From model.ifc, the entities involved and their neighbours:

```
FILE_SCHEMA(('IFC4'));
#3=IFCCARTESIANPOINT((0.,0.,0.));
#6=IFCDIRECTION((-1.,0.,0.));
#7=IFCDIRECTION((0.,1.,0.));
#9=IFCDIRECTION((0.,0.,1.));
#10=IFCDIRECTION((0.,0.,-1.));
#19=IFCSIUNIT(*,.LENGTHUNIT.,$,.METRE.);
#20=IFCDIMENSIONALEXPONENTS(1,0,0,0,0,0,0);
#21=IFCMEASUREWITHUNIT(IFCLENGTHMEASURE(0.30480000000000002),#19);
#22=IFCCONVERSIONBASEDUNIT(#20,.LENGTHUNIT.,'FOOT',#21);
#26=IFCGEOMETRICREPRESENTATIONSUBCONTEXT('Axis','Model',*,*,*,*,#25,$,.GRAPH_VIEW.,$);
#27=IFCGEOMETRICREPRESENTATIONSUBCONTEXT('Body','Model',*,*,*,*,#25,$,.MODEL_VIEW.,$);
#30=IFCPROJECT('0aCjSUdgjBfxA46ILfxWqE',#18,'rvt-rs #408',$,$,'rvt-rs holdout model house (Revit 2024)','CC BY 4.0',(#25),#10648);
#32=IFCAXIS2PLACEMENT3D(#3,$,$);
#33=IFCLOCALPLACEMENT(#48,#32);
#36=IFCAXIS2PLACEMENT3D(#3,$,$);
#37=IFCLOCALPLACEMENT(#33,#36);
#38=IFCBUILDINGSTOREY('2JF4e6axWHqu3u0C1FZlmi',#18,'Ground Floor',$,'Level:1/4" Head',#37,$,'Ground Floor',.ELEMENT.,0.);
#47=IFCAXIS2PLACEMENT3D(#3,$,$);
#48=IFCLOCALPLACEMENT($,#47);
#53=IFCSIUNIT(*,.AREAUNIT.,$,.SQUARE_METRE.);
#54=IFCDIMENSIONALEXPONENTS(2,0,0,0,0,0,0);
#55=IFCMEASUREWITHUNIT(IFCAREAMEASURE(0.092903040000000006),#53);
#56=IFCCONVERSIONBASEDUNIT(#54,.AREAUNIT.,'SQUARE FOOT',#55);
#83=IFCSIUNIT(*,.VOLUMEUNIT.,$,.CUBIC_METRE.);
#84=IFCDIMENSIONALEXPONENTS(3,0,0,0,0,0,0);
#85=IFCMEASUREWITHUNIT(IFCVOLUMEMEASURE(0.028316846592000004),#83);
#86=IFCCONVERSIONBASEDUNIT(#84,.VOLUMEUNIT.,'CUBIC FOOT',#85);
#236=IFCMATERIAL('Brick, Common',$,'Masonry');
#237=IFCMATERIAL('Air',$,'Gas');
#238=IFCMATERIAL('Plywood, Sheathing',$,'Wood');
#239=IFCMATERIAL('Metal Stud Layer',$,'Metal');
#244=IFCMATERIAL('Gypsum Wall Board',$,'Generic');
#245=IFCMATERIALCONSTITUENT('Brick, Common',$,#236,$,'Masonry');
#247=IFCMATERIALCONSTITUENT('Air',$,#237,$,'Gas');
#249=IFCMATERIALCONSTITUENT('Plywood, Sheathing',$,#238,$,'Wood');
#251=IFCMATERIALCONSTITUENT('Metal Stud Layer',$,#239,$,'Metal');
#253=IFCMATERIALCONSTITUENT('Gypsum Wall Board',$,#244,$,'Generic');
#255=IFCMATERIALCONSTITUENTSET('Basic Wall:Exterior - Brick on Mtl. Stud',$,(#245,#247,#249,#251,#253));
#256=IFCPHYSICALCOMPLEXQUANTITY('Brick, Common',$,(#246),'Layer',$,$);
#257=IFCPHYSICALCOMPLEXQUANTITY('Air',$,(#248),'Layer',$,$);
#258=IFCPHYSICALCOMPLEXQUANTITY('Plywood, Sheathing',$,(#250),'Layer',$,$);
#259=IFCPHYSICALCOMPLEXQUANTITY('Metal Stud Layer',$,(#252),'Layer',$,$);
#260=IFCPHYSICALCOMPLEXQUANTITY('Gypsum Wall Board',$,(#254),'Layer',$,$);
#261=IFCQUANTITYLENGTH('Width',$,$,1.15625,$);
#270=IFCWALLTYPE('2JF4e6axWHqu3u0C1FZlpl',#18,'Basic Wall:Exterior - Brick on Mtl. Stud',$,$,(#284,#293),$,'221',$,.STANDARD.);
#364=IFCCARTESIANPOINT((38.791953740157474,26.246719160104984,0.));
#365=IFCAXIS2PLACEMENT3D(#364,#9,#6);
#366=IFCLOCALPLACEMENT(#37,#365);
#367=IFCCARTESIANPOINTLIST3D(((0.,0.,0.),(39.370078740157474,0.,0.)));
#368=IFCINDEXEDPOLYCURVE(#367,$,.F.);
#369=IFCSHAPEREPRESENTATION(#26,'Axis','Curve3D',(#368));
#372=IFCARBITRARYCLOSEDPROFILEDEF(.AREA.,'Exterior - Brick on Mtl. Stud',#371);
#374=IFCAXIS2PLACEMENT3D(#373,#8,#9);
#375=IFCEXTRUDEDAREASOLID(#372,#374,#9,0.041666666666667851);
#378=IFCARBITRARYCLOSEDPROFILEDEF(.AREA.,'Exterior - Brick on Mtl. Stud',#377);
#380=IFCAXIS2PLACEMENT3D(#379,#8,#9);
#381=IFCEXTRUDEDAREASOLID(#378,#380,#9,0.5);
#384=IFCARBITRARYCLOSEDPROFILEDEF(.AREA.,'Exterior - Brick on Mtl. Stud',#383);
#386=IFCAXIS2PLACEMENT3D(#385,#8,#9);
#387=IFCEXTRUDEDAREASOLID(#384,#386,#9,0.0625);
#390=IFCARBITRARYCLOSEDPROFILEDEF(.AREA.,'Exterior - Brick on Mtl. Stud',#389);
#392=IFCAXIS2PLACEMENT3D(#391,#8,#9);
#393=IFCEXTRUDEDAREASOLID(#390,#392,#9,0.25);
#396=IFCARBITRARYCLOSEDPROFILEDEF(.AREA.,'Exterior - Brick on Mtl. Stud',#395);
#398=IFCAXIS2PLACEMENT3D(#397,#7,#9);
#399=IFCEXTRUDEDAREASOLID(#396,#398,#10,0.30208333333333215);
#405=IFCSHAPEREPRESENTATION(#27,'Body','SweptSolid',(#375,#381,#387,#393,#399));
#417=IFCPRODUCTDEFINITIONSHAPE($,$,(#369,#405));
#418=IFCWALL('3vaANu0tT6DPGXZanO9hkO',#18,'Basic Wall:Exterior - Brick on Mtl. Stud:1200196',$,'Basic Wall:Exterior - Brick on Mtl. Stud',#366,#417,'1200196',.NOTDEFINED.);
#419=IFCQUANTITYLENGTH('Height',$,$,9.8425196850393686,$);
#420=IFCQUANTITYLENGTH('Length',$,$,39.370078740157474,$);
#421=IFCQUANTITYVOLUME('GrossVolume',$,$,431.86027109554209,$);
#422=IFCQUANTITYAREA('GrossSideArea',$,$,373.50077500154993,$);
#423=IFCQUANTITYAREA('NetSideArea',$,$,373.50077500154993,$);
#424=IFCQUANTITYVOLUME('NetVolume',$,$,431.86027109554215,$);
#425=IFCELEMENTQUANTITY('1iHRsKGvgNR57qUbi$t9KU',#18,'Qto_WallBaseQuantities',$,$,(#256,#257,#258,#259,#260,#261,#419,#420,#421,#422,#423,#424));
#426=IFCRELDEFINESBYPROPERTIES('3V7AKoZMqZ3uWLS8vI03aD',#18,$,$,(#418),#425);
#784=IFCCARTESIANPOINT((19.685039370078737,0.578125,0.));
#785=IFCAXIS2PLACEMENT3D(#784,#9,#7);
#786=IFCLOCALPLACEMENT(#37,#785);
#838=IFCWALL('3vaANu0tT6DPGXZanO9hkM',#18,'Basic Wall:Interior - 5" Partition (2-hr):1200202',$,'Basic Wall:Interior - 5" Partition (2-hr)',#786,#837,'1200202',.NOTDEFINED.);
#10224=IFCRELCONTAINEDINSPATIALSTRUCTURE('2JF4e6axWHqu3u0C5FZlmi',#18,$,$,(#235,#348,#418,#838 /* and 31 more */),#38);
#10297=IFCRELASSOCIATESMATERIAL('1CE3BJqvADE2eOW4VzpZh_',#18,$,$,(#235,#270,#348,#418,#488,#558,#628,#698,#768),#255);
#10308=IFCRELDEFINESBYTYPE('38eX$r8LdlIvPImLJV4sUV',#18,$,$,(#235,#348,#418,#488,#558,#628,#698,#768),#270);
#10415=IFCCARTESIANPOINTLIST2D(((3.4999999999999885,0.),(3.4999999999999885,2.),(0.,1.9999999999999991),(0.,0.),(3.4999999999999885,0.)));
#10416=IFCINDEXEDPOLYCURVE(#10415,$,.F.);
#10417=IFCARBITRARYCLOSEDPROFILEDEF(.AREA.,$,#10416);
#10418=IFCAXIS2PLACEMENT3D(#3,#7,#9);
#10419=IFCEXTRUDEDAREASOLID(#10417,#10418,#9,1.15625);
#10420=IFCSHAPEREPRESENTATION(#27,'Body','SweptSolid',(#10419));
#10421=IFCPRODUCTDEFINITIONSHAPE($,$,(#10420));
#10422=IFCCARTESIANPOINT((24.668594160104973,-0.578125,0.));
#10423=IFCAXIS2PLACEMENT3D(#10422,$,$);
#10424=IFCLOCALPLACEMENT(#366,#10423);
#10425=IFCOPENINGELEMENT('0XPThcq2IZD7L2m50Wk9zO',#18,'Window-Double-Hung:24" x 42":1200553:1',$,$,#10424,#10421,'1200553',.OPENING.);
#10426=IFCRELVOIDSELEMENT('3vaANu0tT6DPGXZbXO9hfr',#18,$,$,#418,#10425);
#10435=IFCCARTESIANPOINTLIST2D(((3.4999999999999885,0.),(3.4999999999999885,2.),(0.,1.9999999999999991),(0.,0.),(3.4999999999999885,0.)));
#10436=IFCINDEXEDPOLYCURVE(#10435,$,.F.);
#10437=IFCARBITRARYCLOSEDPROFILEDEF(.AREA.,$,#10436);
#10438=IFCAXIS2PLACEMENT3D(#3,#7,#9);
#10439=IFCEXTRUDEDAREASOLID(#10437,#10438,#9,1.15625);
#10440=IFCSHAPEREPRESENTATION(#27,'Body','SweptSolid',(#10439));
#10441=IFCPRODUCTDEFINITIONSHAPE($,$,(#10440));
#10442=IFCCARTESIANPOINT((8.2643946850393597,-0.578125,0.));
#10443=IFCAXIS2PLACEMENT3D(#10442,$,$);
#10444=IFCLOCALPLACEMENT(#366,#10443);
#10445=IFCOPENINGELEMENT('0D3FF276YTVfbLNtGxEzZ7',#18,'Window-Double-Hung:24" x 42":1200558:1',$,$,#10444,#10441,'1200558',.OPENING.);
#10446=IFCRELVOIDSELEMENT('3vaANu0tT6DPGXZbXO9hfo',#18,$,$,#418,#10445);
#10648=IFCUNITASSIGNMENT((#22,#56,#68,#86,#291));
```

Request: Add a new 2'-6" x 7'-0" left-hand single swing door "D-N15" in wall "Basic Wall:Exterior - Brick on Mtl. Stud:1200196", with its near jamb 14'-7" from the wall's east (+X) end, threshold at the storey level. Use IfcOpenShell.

```python
import numpy as np
import ifcopenshell
import ifcopenshell.api.feature
import ifcopenshell.api.geometry
import ifcopenshell.api.pset
import ifcopenshell.api.root
import ifcopenshell.api.spatial
import ifcopenshell.geom
import ifcopenshell.util.element
import ifcopenshell.util.placement
import ifcopenshell.util.representation
import ifcopenshell.util.shape
import ifcopenshell.util.unit

model = ifcopenshell.open("model.ifc")
unit_scale = ifcopenshell.util.unit.calculate_unit_scale(model)
area_scale = ifcopenshell.util.unit.calculate_unit_scale(model, "AREAUNIT")
volume_scale = ifcopenshell.util.unit.calculate_unit_scale(model, "VOLUMEUNIT")
settings = ifcopenshell.geom.settings()


def volume(element):
    """Net volume in cubic metres, openings subtracted."""
    shape = ifcopenshell.geom.create_shape(settings, element)
    return ifcopenshell.util.shape.get_volume(shape.geometry)


wall = model.by_guid("3vaANu0tT6DPGXZanO9hkO")
storey = ifcopenshell.util.element.get_container(wall, ifc_class="IfcBuildingStorey")
context = ifcopenshell.util.representation.get_context(model, "Model", "Body", "MODEL_VIEW")
before = volume(wall)

width, height, from_end, sill = 0.762, 2.1336, 4.445, 0.0  # metres

# The wall runs along its own X axis, and the end named is its -X end.
wall_shape = ifcopenshell.geom.create_shape(settings, wall)
x, y, z = ifcopenshell.util.shape.get_vertices(wall_shape.geometry).T
start = x.min() + from_end
face, thickness = float(y.min()), float(y.max() - y.min())
wall_matrix = ifcopenshell.util.placement.get_local_placement(wall.ObjectPlacement)
level = ifcopenshell.util.placement.get_local_placement(storey.ObjectPlacement)[2, 3]


def in_wall(x, y):
    """Placement at x, y metres in the wall's axes, at sill height."""
    matrix = wall_matrix.copy()
    matrix[:, 3] = wall_matrix @ np.array([x / unit_scale, y / unit_scale, 0.0, 1.0])
    matrix[2, 3] = level + sill / unit_scale
    return matrix


# Opening: a box that overshoots both wall faces by 50 mm.
opening = ifcopenshell.api.root.create_entity(model, ifc_class="IfcOpeningElement", predefined_type="OPENING")
box = ifcopenshell.api.geometry.add_wall_representation(
    model, context=context, length=width, height=height, thickness=thickness + 0.1
)
ifcopenshell.api.geometry.assign_representation(model, product=opening, representation=box)
ifcopenshell.api.geometry.edit_object_placement(model, product=opening, matrix=in_wall(start, face - 0.05), is_si=False)
ifcopenshell.api.feature.add_feature(model, feature=opening, element=wall)

door = ifcopenshell.api.root.create_entity(model, ifc_class="IfcDoor", name="D-N15", predefined_type="DOOR")
door.OverallWidth, door.OverallHeight = width / unit_scale, height / unit_scale
door.OperationType = "SINGLE_SWING_LEFT"
body = ifcopenshell.api.geometry.add_door_representation(
    model,
    context=context,
    overall_width=door.OverallWidth,
    overall_height=door.OverallHeight,
    operation_type="SINGLE_SWING_LEFT",
    lining_properties={"LiningDepth": thickness / unit_scale, "ThresholdDepth": thickness / unit_scale},
)
ifcopenshell.api.geometry.assign_representation(model, product=door, representation=body)
ifcopenshell.api.spatial.assign_container(model, products=[door], relating_structure=storey)
ifcopenshell.api.feature.add_filling(model, opening=opening, element=door)

# The lining spans the wall, so the door starts at the wall face.
ifcopenshell.api.geometry.edit_object_placement(model, product=door, matrix=in_wall(start, face), is_si=False)

after = volume(wall)

# Update the wall's stored quantities.
qto = model.by_id(ifcopenshell.util.element.get_pset(wall, "Qto_WallBaseQuantities", should_inherit=False)["id"])
ifcopenshell.api.pset.edit_qto(model, qto=qto, properties={
    "NetSideArea": after / thickness / area_scale,
    "NetVolume": after / volume_scale,
})

print(f"wall volume {before:.3f} -> {after:.3f} m3")

model.write("model_edited.ifc")
```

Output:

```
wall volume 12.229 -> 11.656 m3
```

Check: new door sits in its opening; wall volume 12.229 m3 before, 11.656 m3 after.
